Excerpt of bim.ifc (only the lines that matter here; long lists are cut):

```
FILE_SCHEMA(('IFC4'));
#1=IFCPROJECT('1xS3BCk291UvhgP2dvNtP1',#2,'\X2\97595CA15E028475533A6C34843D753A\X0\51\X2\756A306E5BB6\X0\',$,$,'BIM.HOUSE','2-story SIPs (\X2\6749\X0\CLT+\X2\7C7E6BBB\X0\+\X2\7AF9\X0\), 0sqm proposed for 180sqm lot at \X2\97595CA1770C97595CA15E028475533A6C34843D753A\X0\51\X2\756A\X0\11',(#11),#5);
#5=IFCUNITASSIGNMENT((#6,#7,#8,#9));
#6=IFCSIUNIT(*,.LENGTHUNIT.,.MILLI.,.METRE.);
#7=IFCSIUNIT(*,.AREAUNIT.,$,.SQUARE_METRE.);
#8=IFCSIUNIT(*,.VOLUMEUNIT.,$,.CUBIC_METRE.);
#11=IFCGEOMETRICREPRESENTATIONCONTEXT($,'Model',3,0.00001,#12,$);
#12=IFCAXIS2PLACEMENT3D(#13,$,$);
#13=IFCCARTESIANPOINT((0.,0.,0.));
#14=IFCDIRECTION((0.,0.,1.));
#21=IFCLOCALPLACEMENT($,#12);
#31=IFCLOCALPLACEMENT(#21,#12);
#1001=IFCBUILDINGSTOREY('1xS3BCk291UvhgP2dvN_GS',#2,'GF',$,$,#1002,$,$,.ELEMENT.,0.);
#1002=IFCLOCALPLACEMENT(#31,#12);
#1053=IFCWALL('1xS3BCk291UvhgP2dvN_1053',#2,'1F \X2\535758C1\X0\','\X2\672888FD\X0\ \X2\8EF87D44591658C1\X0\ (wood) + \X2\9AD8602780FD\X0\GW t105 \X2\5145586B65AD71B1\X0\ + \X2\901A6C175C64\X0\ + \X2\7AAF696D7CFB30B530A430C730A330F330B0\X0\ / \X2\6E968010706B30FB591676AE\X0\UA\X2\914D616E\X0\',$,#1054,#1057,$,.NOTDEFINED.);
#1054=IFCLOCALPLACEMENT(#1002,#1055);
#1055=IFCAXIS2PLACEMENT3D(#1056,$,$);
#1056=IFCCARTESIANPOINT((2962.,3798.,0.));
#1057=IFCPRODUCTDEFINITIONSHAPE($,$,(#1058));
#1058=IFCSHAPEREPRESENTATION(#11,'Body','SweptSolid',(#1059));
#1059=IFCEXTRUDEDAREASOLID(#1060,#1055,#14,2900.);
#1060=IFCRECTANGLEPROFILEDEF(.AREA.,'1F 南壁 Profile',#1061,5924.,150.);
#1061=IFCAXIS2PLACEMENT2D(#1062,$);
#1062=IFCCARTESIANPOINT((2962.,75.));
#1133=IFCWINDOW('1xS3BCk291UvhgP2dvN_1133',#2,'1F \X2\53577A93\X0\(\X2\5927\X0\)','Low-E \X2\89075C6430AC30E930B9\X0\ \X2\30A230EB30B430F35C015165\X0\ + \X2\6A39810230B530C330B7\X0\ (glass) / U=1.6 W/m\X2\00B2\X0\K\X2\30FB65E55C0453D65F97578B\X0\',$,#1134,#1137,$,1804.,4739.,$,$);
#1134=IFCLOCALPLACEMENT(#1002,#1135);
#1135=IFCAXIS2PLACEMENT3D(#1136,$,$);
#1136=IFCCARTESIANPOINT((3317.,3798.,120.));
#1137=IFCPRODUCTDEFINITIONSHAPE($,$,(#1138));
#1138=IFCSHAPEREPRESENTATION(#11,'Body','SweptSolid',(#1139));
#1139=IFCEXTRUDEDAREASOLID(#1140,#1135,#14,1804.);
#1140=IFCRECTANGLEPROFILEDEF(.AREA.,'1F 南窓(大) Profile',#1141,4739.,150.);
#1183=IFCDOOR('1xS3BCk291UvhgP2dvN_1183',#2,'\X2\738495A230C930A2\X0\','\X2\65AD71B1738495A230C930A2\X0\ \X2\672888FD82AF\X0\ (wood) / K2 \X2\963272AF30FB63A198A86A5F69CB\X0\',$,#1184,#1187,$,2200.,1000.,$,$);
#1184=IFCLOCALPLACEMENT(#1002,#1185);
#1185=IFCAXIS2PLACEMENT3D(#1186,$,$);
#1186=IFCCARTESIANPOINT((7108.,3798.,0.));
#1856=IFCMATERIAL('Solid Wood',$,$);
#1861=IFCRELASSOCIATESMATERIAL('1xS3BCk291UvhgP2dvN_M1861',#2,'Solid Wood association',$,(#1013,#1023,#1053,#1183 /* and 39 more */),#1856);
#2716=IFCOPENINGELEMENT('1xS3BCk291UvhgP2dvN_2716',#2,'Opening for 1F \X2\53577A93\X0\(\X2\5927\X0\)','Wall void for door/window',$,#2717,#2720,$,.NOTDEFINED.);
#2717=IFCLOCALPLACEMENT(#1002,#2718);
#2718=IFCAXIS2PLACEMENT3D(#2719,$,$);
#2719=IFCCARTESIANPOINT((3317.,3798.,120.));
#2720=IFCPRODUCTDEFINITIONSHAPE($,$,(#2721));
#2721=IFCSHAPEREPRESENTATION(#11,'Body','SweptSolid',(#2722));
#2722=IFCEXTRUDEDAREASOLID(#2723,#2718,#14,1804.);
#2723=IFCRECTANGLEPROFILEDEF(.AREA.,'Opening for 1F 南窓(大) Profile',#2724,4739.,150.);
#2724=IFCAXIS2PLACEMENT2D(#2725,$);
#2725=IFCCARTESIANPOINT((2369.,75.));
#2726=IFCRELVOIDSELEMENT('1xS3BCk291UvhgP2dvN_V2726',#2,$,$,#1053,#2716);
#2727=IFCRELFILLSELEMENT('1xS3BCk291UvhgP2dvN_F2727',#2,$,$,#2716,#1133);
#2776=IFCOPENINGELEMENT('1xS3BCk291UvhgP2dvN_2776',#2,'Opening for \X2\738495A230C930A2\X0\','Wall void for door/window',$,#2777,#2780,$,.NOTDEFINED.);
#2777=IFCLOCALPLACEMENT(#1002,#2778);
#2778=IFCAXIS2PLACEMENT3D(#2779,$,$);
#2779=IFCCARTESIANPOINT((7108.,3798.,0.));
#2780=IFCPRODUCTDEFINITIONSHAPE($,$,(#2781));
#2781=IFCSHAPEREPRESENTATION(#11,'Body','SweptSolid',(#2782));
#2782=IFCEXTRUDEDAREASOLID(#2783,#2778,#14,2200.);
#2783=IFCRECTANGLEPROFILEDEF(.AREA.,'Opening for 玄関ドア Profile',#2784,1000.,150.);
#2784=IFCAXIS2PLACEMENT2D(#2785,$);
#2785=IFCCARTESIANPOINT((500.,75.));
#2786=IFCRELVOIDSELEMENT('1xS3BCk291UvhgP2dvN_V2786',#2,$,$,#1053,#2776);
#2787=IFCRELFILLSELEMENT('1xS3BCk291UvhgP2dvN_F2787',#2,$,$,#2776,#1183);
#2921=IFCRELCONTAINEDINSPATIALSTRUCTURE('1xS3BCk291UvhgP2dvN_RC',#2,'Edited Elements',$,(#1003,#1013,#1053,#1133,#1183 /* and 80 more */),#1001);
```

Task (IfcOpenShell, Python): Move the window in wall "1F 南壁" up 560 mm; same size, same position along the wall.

```python
import numpy as np
import ifcopenshell
import ifcopenshell.api.geometry
import ifcopenshell.util.placement
import ifcopenshell.util.unit

model = ifcopenshell.open("bim.ifc")
unit_scale = ifcopenshell.util.unit.calculate_unit_scale(model)

window = model.by_guid("1xS3BCk291UvhgP2dvN_1133")
opening = window.FillsVoids[0].RelatingOpeningElement
dz = 0.56 / unit_scale

shift = np.array([0.0, 0.0, dz])
# The window is not placed relative to its opening, so move both.
for product in (opening, window):
    matrix = ifcopenshell.util.placement.get_local_placement(product.ObjectPlacement)
    matrix[:3, 3] += shift
    ifcopenshell.api.geometry.edit_object_placement(model, product=product, matrix=matrix, is_si=False)

print(f"moved by {dz * unit_scale:+.3f} m")

model.write("bim-out.ifc")
```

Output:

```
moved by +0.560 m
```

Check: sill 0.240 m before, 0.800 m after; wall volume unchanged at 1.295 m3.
